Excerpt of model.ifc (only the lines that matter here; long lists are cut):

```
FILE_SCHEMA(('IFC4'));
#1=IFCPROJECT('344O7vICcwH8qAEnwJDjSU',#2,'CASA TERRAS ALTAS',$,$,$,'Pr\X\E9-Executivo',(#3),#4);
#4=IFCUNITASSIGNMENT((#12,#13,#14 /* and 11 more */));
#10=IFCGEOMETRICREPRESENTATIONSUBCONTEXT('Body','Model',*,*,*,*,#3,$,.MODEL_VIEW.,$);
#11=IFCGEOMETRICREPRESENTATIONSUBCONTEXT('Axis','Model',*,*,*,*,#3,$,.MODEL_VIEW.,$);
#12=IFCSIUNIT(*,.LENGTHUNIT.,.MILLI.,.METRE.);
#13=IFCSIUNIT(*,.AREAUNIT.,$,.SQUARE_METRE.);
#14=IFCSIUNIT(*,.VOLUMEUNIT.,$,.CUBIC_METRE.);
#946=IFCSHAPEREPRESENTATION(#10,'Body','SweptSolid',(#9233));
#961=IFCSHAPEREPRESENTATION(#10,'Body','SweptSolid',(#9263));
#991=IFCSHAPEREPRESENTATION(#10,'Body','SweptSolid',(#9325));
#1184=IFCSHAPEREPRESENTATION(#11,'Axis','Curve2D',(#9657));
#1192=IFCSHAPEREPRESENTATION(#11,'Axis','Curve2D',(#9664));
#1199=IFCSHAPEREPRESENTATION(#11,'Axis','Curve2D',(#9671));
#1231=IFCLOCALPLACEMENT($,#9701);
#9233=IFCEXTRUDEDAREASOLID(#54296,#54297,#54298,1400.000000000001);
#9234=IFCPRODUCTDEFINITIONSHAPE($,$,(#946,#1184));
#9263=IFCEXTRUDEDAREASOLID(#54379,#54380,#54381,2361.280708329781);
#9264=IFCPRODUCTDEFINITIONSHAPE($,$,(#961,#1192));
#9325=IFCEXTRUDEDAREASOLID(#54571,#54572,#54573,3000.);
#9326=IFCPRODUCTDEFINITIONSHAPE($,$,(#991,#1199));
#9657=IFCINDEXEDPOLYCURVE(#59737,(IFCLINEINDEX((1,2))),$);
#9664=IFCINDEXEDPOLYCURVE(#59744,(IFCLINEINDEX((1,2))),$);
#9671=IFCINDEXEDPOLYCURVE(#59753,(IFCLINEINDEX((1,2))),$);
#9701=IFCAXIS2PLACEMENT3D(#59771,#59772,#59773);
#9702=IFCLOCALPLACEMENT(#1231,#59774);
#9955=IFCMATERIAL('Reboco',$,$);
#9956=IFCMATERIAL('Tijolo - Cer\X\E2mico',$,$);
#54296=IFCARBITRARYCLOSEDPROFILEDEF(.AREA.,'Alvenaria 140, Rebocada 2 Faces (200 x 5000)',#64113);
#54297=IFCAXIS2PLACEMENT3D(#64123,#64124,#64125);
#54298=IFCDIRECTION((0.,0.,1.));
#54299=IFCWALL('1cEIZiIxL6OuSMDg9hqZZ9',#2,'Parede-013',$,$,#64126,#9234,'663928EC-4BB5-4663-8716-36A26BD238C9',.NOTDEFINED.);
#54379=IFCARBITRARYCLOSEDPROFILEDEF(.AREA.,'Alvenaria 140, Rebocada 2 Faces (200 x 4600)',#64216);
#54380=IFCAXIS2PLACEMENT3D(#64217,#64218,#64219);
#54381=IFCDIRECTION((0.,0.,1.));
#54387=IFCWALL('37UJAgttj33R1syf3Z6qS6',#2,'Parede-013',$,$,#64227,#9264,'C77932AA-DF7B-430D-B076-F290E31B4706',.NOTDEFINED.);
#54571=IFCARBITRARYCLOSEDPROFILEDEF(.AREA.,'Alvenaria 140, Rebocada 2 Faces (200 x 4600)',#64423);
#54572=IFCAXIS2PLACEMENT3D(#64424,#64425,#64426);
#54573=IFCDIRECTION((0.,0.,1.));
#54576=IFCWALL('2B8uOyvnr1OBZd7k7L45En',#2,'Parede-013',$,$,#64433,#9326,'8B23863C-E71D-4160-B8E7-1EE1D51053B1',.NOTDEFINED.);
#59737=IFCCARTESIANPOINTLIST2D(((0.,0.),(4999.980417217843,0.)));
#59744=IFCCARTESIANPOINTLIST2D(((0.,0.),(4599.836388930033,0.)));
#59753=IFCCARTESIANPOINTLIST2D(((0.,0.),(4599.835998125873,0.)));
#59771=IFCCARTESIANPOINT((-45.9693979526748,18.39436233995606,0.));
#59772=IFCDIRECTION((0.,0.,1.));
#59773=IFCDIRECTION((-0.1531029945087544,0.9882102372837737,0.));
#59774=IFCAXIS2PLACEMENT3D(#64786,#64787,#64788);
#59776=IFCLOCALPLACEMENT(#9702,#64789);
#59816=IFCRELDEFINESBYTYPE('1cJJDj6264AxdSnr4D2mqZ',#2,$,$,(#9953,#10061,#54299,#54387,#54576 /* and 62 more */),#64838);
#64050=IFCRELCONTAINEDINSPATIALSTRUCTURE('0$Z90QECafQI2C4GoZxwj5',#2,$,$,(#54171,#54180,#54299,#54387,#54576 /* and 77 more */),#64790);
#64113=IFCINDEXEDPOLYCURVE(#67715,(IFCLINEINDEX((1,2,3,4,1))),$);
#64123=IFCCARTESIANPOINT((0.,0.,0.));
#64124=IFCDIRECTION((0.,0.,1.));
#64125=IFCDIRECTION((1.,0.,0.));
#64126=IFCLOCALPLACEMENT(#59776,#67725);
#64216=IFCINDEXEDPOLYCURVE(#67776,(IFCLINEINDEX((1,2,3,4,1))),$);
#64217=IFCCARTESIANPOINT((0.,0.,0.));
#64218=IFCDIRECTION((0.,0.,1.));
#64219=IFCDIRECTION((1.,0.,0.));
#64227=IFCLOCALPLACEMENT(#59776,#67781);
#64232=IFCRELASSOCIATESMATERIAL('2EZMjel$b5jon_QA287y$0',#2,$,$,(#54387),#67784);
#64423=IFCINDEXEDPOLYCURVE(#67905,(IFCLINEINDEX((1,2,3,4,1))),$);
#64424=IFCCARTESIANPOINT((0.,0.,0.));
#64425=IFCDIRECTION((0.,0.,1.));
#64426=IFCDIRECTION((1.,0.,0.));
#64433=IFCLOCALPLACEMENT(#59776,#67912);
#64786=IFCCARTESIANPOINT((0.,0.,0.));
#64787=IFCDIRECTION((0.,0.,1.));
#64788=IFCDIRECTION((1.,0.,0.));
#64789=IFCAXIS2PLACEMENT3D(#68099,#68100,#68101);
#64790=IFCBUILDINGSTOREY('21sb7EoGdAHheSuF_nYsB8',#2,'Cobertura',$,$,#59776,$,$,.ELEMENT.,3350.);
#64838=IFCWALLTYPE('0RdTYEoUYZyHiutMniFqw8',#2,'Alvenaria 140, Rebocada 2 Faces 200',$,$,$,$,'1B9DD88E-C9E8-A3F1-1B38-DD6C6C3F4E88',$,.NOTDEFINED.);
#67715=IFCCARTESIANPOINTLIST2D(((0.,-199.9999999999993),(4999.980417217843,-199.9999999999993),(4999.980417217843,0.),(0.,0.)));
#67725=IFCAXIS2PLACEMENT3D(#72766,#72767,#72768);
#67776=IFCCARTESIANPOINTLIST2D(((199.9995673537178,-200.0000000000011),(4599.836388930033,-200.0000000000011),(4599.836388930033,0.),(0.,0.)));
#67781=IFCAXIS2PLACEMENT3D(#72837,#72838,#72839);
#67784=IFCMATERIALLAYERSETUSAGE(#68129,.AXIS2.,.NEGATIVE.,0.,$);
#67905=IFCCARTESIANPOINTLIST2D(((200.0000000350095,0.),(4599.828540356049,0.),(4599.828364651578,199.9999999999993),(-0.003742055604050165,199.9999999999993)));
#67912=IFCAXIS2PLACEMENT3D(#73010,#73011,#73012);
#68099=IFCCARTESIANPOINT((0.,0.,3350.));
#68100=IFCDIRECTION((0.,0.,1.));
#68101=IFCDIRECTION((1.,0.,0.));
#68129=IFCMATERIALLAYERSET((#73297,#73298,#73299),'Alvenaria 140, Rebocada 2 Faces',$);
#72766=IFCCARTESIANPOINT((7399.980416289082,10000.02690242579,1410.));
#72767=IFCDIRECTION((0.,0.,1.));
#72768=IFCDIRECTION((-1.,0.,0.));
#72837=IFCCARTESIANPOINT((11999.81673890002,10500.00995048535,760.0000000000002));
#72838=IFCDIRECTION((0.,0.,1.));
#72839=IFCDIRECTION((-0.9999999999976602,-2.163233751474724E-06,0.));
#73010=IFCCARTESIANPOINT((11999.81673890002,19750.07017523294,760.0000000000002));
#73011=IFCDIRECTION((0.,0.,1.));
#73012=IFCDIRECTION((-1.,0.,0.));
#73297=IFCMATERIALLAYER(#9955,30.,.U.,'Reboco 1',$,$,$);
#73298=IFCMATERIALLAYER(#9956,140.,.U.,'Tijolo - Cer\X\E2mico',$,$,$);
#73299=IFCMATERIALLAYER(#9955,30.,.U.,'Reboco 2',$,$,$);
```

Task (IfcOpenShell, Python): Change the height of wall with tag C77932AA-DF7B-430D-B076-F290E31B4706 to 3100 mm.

```python
import ifcopenshell
import ifcopenshell.geom
import ifcopenshell.util.representation
import ifcopenshell.util.shape

model = ifcopenshell.open("model.ifc")
settings = ifcopenshell.geom.settings()


def volume(element):
    """Net volume in cubic metres, openings subtracted."""
    shape = ifcopenshell.geom.create_shape(settings, element)
    return ifcopenshell.util.shape.get_volume(shape.geometry)


wall = model.by_id(54387)
before = volume(wall)

body = ifcopenshell.util.representation.get_representation(wall, "Model", "Body")
solid = body.Items[0]
old_height = solid.Depth
solid.Depth = 3100.0
after = volume(wall)

print(f"height {old_height:g} -> {solid.Depth:g}, volume {before:.3f} -> {after:.3f} m3")

model.write("model_edited.ifc")
```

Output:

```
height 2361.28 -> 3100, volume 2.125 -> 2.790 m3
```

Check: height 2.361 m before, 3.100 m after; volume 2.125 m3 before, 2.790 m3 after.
